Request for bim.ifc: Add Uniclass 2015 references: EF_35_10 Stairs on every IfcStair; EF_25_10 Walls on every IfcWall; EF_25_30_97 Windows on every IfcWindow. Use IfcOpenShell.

First a look at what the model holds.

```python
import ifcopenshell

model = ifcopenshell.open("bim.ifc")
print(model.schema)
print("classifications:", [c.Name for c in model.by_type("IfcClassification")])
for ifc_class in ("IfcDoor", "IfcRoof", "IfcStair", "IfcWall", "IfcWindow"):
    print(ifc_class, len(model.by_type(ifc_class)))
```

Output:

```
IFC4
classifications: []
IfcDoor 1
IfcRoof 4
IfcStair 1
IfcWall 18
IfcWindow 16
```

```python
import ifcopenshell
import ifcopenshell.api.classification

model = ifcopenshell.open("bim.ifc")

system = ifcopenshell.api.classification.add_classification(model, classification="Uniclass 2015")

codes = {
    "IfcStair": ("EF_35_10", "Stairs"),
    "IfcWall": ("EF_25_10", "Walls"),
    "IfcWindow": ("EF_25_30_97", "Windows"),
}
for ifc_class, (code, name) in codes.items():
    products = model.by_type(ifc_class)
    ifcopenshell.api.classification.add_reference(
        model, products=products, classification=system, identification=code, name=name
    )
    print(code, len(products))

model.write("bim_v2.ifc")
```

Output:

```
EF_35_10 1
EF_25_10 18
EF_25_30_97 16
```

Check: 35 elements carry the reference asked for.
